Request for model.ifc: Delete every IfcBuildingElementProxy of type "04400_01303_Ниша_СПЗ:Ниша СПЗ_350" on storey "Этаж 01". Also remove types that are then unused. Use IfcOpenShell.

First a look at what the model holds.

```python
import ifcopenshell
import ifcopenshell.util.element

model = ifcopenshell.open("model.ifc")
print(model.schema)
storey = next(s for s in model.by_type("IfcBuildingStorey") if s.Name == "Этаж 01")
proxies = [e for e in ifcopenshell.util.element.get_decomposition(storey) if e.is_a("IfcBuildingElementProxy")]
seen = {}
for e in proxies:
    element_type = ifcopenshell.util.element.get_type(e)
    name = element_type.Name if element_type not in (None, e) else None
    seen[name] = seen.get(name, 0) + 1
for name, count in sorted(seen.items(), key=str):
    print(count, "x", name)
```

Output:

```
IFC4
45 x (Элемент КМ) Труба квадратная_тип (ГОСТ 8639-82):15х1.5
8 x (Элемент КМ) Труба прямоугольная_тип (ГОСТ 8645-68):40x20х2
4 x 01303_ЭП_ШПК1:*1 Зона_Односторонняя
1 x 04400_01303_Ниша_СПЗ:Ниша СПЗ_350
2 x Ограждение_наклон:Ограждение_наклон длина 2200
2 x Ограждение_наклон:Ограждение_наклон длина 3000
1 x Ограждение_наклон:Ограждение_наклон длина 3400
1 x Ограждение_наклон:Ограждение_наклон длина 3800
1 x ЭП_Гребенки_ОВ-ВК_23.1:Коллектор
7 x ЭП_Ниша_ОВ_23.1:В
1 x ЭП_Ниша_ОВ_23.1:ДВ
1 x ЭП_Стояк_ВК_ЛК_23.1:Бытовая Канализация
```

```python
import ifcopenshell
import ifcopenshell.api.root
import ifcopenshell.util.element

model = ifcopenshell.open("model.ifc")

storey = next(s for s in model.by_type("IfcBuildingStorey") if s.Name == "Этаж 01")
proxies = [e for e in ifcopenshell.util.element.get_decomposition(storey) if e.is_a("IfcBuildingElementProxy")]
targets = [e for e in proxies if (t := ifcopenshell.util.element.get_type(e)) not in (None, e) and t.Name == "04400_01303_Ниша_СПЗ:Ниша СПЗ_350"]
types = {ifcopenshell.util.element.get_type(e) for e in targets} - {None, *targets}

for e in targets:
    ifcopenshell.api.root.remove_product(model, product=e)
print(len(targets), "removed")

unused = [t for t in types if not ifcopenshell.util.element.get_types(t)]
for t in unused:
    ifcopenshell.api.root.remove_product(model, product=t)
print(len(unused), "unused types removed")

model.write("model_updated.ifc")
```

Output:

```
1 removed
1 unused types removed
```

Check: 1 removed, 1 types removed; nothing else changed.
